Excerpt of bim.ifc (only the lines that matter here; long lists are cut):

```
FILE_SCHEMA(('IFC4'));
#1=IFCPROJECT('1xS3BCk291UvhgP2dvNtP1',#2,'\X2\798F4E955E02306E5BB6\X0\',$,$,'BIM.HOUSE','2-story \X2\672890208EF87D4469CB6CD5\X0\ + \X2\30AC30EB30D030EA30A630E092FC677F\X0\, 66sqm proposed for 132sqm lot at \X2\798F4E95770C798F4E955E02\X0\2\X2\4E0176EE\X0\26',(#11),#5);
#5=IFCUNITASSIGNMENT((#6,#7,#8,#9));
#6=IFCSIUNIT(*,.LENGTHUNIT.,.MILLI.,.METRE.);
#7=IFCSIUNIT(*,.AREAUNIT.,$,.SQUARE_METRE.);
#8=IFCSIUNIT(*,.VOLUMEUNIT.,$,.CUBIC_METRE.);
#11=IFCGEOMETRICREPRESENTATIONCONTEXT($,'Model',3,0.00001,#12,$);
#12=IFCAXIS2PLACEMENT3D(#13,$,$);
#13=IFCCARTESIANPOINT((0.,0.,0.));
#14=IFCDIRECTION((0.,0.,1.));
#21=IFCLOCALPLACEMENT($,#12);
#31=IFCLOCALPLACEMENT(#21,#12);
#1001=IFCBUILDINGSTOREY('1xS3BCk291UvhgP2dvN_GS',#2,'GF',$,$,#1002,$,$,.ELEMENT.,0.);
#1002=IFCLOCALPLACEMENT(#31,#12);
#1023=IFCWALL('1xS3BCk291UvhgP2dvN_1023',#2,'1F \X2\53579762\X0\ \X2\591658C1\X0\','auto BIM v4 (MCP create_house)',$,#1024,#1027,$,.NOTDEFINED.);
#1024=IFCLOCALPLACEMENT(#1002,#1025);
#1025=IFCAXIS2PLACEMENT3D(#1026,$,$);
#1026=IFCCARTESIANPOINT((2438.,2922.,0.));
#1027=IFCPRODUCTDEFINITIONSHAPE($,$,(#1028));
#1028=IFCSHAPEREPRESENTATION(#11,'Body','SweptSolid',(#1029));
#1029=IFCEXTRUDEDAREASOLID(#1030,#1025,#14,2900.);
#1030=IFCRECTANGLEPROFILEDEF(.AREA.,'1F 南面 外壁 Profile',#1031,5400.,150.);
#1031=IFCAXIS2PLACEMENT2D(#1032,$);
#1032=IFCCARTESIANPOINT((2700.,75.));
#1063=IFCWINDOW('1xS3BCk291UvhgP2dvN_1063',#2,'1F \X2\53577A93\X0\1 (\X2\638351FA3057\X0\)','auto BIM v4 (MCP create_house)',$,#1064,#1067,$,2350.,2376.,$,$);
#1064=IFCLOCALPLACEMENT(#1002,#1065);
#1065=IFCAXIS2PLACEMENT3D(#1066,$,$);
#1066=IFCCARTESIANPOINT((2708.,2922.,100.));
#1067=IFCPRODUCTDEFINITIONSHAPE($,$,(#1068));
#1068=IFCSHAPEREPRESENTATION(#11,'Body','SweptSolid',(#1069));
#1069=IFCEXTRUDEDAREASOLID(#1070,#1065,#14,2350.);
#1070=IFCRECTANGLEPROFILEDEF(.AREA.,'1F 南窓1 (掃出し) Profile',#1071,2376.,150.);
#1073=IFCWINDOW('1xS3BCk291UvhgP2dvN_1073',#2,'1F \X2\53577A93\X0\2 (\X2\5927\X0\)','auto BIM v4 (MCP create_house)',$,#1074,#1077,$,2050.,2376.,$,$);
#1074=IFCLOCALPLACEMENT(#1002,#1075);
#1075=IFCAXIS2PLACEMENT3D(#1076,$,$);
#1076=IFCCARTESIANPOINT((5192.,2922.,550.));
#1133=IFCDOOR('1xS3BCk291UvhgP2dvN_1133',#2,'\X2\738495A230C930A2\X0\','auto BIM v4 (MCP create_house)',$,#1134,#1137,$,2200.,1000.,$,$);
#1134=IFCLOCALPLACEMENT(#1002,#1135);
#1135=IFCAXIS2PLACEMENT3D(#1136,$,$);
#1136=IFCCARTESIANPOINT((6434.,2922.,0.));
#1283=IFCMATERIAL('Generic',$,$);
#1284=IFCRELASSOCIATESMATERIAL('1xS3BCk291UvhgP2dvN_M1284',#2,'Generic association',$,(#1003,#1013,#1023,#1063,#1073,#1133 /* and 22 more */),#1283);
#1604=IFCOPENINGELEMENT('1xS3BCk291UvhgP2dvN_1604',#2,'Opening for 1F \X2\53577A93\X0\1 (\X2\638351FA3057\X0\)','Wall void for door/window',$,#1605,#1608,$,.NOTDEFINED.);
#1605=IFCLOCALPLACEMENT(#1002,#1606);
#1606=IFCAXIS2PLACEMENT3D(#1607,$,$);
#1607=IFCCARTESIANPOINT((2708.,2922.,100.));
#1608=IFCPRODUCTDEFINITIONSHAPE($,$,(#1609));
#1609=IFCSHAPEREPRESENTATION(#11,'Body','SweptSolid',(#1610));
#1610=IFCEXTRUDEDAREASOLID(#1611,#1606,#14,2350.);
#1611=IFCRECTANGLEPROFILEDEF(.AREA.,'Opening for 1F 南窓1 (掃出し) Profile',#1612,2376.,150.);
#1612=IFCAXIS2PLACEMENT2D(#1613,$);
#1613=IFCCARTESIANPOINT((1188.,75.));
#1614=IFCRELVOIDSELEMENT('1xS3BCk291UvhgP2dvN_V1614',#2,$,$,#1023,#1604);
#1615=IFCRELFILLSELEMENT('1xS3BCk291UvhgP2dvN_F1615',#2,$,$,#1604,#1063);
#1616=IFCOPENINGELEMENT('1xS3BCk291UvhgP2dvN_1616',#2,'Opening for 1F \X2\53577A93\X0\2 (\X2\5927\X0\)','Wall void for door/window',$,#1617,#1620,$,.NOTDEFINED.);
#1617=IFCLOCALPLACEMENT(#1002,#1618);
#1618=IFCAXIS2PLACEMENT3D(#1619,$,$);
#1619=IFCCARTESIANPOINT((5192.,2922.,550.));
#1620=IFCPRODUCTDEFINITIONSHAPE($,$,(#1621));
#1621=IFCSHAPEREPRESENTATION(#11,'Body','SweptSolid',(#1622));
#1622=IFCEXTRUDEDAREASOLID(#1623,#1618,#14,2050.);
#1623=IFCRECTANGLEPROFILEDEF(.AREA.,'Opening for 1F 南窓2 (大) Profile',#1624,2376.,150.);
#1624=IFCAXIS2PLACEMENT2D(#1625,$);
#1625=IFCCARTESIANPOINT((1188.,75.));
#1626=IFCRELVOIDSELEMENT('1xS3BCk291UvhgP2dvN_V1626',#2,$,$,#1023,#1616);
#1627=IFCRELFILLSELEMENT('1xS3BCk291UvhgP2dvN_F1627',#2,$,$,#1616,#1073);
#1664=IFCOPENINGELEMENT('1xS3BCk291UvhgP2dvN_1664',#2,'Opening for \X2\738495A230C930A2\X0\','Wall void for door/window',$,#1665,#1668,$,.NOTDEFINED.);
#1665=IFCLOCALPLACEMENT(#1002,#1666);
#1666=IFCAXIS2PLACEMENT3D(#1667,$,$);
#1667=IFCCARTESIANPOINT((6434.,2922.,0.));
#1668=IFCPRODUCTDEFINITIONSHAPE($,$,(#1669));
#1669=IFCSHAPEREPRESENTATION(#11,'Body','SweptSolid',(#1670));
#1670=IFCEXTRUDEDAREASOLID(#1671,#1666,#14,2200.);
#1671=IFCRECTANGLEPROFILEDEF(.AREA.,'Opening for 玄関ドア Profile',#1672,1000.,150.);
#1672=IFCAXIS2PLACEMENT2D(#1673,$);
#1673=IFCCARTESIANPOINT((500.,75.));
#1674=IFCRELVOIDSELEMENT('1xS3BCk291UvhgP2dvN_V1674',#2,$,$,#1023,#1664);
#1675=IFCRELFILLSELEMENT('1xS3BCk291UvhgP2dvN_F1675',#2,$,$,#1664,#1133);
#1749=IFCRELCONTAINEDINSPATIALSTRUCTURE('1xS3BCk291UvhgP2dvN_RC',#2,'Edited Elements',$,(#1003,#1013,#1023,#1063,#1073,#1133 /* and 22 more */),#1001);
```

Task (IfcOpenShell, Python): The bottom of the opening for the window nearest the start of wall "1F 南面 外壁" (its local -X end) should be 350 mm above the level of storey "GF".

```python
import numpy as np
import ifcopenshell
import ifcopenshell.api.geometry
import ifcopenshell.geom
import ifcopenshell.util.element
import ifcopenshell.util.placement
import ifcopenshell.util.shape
import ifcopenshell.util.unit

model = ifcopenshell.open("bim.ifc")
unit_scale = ifcopenshell.util.unit.calculate_unit_scale(model)

window = model.by_id(1063)
opening = window.FillsVoids[0].RelatingOpeningElement
storey = ifcopenshell.util.element.get_container(window, ifc_class="IfcBuildingStorey")
level = ifcopenshell.util.placement.get_local_placement(storey.ObjectPlacement)[2, 3]

# The opening's origin need not be at the sill, so measure its lowest point.
shape = ifcopenshell.geom.create_shape(ifcopenshell.geom.settings(), opening)
bottom = ifcopenshell.util.shape.get_shape_bottom_elevation(shape, shape.geometry) / unit_scale
dz = level + 350.0 - bottom

shift = np.array([0.0, 0.0, dz])
# The window is not placed relative to its opening, so move both.
for product in (opening, window):
    matrix = ifcopenshell.util.placement.get_local_placement(product.ObjectPlacement)
    matrix[:3, 3] += shift
    ifcopenshell.api.geometry.edit_object_placement(model, product=product, matrix=matrix, is_si=False)

print(f"moved by {dz * unit_scale:+.3f} m")

model.write("bim_v2.ifc")
```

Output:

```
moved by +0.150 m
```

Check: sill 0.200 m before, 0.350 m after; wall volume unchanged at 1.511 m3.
